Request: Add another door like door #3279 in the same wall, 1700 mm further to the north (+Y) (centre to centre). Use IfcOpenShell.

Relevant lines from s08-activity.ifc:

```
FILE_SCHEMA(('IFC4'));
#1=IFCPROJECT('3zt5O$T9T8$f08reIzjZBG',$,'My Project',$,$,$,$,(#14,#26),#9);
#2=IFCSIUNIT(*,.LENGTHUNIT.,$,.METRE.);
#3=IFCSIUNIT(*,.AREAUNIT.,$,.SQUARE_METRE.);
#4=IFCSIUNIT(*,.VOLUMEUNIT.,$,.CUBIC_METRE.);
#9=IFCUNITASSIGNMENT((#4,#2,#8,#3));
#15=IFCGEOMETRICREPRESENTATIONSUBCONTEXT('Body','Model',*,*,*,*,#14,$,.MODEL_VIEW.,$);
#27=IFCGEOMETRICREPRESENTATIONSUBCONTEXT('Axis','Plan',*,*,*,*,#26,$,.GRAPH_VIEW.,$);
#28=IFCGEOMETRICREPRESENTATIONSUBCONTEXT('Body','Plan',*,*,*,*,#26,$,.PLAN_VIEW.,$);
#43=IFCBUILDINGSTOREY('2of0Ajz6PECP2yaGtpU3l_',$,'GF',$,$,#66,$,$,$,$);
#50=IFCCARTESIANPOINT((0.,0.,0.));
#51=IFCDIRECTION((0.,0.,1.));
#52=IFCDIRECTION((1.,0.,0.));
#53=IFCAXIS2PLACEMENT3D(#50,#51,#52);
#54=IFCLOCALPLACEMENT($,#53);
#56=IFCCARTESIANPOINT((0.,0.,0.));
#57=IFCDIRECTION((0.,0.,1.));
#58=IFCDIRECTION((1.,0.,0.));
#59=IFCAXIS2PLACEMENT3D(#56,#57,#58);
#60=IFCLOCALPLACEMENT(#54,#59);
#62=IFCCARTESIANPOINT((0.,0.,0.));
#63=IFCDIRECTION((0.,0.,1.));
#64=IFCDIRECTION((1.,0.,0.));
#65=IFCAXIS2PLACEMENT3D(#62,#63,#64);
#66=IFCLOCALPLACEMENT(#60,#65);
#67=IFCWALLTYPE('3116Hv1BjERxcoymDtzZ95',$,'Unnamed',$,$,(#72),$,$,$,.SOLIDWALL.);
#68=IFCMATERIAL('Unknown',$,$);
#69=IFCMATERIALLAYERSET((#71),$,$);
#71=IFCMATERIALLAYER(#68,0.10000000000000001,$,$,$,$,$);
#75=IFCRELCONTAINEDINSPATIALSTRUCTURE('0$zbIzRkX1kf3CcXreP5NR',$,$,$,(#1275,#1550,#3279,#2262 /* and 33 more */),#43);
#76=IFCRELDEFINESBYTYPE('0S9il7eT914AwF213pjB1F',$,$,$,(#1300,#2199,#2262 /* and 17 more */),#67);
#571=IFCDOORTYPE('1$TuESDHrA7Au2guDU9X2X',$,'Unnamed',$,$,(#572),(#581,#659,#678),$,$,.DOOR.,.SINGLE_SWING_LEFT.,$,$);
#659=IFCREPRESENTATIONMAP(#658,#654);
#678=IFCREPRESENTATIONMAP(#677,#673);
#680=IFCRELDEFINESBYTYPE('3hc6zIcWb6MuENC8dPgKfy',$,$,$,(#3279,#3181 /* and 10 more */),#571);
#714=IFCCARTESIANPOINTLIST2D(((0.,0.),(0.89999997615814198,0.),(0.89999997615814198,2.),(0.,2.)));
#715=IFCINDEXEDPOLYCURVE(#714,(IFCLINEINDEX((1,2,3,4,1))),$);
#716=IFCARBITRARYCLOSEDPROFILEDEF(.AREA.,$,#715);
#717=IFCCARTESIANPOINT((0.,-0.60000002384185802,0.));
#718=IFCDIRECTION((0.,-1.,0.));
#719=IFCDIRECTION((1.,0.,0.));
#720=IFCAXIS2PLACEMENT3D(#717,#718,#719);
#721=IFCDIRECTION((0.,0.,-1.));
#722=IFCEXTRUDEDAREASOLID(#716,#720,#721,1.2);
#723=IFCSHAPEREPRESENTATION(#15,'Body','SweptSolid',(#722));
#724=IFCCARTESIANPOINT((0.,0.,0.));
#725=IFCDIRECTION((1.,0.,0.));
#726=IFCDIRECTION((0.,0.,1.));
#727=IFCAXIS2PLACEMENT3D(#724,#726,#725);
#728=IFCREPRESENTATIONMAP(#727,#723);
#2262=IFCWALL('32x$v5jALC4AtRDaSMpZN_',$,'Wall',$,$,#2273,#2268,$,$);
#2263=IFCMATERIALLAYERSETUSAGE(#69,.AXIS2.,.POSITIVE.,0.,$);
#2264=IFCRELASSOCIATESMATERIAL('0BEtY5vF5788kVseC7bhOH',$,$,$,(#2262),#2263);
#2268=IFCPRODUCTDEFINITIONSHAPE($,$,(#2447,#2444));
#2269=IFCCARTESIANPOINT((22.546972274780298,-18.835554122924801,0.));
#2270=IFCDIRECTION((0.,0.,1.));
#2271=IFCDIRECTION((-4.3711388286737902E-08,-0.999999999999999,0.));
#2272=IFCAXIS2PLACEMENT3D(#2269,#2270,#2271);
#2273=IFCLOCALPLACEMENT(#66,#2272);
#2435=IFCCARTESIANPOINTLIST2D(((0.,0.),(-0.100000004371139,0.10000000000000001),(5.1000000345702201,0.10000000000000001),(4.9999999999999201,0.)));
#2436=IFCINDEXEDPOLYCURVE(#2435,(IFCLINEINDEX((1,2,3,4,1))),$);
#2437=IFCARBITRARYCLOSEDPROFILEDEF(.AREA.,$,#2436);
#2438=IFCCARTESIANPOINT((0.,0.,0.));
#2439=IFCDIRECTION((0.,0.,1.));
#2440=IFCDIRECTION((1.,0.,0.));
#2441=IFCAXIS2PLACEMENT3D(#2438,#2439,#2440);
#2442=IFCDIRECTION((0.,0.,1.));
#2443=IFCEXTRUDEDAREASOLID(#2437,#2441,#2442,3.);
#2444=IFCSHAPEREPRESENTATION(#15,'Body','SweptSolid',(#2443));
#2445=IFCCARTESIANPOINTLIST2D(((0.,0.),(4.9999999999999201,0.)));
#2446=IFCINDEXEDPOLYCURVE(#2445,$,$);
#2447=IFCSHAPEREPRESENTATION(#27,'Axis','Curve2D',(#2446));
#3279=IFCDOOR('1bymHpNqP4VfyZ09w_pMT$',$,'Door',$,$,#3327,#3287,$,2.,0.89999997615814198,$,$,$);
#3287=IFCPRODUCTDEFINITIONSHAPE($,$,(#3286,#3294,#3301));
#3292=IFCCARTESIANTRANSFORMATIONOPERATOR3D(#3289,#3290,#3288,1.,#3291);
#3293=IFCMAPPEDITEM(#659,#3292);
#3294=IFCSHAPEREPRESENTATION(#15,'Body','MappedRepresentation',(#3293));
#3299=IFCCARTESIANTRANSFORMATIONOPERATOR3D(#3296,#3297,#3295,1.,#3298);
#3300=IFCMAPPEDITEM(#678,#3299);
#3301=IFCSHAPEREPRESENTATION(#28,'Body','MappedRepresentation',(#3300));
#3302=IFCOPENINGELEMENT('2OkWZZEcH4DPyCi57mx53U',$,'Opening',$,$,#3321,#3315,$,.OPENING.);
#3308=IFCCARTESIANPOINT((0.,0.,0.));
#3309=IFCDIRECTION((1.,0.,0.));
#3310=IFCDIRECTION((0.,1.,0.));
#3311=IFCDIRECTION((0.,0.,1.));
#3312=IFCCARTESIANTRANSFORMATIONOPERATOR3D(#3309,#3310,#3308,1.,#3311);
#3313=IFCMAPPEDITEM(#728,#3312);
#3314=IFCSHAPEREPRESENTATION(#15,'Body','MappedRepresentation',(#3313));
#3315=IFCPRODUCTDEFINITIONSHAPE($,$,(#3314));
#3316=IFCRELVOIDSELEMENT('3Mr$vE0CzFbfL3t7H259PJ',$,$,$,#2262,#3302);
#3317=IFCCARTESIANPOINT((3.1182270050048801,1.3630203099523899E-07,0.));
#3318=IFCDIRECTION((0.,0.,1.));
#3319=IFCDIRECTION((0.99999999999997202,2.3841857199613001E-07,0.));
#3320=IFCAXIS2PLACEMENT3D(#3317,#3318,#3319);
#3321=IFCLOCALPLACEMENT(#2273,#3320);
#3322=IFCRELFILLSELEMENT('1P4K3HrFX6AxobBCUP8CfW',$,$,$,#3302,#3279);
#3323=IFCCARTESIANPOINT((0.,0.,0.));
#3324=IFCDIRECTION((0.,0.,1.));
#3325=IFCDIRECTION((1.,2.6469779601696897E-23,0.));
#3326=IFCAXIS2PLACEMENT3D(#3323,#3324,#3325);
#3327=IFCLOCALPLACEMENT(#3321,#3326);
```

```python
import ifcopenshell
import ifcopenshell.api.feature
import ifcopenshell.api.geometry
import ifcopenshell.api.root
import ifcopenshell.geom
import ifcopenshell.util.element
import ifcopenshell.util.placement
import ifcopenshell.util.shape
import ifcopenshell.util.unit

model = ifcopenshell.open("s08-activity.ifc")
unit_scale = ifcopenshell.util.unit.calculate_unit_scale(model)
settings = ifcopenshell.geom.settings()


def volume(element):
    """Net volume in cubic metres, openings subtracted."""
    shape = ifcopenshell.geom.create_shape(settings, element)
    return ifcopenshell.util.shape.get_volume(shape.geometry)


door = model.by_guid("1bymHpNqP4VfyZ09w_pMT$")
opening = door.FillsVoids[0].RelatingOpeningElement
wall = opening.VoidsElements[0].RelatingBuildingElement
before = volume(wall)
shift = ifcopenshell.util.placement.get_local_placement(wall.ObjectPlacement)[:3, 0] * -1.7 / unit_scale

# copy_class copies the void relationship, type, container and properties, but no geometry.
new_opening = ifcopenshell.api.root.copy_class(model, product=opening)
new_opening.Representation = ifcopenshell.util.element.copy_deep(
    model, opening.Representation, exclude=["IfcGeometricRepresentationContext", "IfcRepresentationMap"]
)
new_door = ifcopenshell.api.root.copy_class(model, product=door)
new_door.Representation = ifcopenshell.util.element.copy_deep(
    model, door.Representation, exclude=["IfcGeometricRepresentationContext", "IfcRepresentationMap"]
)
ifcopenshell.api.feature.add_filling(model, opening=new_opening, element=new_door)

for old, new in ((opening, new_opening), (door, new_door)):
    matrix = ifcopenshell.util.placement.get_local_placement(old.ObjectPlacement)
    matrix[:3, 3] += shift
    ifcopenshell.api.geometry.edit_object_placement(model, product=new, matrix=matrix, is_si=False)

after = volume(wall)

print(f"wall volume {before:.3f} -> {after:.3f} m3")

model.write("s08-activity_v2.ifc")
```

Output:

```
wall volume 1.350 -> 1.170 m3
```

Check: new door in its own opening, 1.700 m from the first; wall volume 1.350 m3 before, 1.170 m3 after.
